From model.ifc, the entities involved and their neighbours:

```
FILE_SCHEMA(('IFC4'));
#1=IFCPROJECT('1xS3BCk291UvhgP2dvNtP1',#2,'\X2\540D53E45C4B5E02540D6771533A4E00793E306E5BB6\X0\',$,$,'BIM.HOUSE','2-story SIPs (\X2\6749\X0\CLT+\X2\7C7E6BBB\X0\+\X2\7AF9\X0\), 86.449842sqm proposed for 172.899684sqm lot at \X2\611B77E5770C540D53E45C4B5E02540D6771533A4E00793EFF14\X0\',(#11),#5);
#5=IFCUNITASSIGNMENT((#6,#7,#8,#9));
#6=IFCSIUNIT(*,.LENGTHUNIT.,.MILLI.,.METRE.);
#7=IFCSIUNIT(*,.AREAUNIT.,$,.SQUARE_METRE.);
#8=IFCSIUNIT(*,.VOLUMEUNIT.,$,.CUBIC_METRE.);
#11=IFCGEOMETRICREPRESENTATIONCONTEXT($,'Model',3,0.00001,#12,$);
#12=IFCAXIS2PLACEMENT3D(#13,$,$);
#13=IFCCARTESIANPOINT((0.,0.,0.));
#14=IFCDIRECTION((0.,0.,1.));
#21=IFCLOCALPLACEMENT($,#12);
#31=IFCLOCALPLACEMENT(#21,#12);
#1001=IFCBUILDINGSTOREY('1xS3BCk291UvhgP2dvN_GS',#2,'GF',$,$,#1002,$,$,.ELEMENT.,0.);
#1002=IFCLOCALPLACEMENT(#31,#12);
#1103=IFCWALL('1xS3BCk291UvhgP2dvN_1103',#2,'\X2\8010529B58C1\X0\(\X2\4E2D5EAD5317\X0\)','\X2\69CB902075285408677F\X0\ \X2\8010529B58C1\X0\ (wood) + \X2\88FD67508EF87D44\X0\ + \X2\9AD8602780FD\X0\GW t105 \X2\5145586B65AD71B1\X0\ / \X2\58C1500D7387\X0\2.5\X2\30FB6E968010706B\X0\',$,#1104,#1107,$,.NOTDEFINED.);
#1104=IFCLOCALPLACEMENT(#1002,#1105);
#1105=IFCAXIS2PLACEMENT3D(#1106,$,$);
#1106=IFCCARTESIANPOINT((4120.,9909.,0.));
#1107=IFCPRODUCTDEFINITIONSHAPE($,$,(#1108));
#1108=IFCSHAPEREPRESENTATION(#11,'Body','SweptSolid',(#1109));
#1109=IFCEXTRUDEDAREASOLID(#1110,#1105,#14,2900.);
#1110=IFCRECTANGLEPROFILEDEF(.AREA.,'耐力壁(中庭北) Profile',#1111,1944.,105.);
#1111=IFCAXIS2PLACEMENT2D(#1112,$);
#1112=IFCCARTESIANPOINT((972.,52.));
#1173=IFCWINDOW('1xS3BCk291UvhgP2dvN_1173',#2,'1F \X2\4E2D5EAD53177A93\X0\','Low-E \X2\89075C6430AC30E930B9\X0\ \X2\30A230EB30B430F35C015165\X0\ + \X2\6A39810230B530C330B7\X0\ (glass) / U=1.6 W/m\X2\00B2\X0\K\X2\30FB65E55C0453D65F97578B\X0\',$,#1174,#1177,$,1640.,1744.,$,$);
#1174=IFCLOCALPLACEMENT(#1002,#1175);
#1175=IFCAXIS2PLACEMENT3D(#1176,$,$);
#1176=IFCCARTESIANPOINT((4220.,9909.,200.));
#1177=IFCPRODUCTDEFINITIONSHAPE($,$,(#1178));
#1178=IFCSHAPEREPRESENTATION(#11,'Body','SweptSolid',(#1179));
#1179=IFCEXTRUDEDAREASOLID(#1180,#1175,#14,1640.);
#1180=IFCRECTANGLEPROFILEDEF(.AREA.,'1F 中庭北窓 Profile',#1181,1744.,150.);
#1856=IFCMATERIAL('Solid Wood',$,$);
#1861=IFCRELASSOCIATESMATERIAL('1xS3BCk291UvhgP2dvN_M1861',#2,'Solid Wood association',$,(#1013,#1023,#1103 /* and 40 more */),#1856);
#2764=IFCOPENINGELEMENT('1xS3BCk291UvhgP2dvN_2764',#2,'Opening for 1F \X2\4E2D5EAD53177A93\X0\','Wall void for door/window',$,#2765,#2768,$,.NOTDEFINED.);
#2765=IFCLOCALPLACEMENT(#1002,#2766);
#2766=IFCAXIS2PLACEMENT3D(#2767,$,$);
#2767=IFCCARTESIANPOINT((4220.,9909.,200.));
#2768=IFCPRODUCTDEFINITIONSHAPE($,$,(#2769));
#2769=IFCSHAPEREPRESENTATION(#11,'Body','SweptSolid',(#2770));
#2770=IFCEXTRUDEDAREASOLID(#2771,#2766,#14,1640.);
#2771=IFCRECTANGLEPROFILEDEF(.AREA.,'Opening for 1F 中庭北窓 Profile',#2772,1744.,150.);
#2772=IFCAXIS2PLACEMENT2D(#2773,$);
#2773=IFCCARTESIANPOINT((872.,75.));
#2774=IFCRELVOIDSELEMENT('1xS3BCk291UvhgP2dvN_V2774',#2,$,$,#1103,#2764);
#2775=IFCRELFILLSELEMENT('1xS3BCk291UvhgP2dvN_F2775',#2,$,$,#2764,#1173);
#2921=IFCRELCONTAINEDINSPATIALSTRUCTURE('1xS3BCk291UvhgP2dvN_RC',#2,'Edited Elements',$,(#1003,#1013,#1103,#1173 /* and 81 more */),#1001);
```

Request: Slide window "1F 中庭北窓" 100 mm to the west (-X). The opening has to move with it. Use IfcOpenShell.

```python
import ifcopenshell
import ifcopenshell.api.geometry
import ifcopenshell.util.placement
import ifcopenshell.util.unit

model = ifcopenshell.open("model.ifc")
unit_scale = ifcopenshell.util.unit.calculate_unit_scale(model)

window = model.by_guid("1xS3BCk291UvhgP2dvN_1173")
opening = window.FillsVoids[0].RelatingOpeningElement
wall = opening.VoidsElements[0].RelatingBuildingElement

wall_matrix = ifcopenshell.util.placement.get_local_placement(wall.ObjectPlacement)
shift = wall_matrix[:3, 0] * -0.1 / unit_scale
before = ifcopenshell.util.placement.get_local_placement(window.ObjectPlacement)[:3, 3].copy()

# The window is not placed relative to its opening, so move both.
for product in (opening, window):
    matrix = ifcopenshell.util.placement.get_local_placement(product.ObjectPlacement)
    matrix[:3, 3] += shift
    ifcopenshell.api.geometry.edit_object_placement(model, product=product, matrix=matrix, is_si=False)

after = ifcopenshell.util.placement.get_local_placement(window.ObjectPlacement)[:3, 3]
print("window moved by", (after - before).round(3) + 0.0)

model.write("model_updated.ifc")
```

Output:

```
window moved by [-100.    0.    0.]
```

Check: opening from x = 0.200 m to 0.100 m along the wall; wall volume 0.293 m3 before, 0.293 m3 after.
